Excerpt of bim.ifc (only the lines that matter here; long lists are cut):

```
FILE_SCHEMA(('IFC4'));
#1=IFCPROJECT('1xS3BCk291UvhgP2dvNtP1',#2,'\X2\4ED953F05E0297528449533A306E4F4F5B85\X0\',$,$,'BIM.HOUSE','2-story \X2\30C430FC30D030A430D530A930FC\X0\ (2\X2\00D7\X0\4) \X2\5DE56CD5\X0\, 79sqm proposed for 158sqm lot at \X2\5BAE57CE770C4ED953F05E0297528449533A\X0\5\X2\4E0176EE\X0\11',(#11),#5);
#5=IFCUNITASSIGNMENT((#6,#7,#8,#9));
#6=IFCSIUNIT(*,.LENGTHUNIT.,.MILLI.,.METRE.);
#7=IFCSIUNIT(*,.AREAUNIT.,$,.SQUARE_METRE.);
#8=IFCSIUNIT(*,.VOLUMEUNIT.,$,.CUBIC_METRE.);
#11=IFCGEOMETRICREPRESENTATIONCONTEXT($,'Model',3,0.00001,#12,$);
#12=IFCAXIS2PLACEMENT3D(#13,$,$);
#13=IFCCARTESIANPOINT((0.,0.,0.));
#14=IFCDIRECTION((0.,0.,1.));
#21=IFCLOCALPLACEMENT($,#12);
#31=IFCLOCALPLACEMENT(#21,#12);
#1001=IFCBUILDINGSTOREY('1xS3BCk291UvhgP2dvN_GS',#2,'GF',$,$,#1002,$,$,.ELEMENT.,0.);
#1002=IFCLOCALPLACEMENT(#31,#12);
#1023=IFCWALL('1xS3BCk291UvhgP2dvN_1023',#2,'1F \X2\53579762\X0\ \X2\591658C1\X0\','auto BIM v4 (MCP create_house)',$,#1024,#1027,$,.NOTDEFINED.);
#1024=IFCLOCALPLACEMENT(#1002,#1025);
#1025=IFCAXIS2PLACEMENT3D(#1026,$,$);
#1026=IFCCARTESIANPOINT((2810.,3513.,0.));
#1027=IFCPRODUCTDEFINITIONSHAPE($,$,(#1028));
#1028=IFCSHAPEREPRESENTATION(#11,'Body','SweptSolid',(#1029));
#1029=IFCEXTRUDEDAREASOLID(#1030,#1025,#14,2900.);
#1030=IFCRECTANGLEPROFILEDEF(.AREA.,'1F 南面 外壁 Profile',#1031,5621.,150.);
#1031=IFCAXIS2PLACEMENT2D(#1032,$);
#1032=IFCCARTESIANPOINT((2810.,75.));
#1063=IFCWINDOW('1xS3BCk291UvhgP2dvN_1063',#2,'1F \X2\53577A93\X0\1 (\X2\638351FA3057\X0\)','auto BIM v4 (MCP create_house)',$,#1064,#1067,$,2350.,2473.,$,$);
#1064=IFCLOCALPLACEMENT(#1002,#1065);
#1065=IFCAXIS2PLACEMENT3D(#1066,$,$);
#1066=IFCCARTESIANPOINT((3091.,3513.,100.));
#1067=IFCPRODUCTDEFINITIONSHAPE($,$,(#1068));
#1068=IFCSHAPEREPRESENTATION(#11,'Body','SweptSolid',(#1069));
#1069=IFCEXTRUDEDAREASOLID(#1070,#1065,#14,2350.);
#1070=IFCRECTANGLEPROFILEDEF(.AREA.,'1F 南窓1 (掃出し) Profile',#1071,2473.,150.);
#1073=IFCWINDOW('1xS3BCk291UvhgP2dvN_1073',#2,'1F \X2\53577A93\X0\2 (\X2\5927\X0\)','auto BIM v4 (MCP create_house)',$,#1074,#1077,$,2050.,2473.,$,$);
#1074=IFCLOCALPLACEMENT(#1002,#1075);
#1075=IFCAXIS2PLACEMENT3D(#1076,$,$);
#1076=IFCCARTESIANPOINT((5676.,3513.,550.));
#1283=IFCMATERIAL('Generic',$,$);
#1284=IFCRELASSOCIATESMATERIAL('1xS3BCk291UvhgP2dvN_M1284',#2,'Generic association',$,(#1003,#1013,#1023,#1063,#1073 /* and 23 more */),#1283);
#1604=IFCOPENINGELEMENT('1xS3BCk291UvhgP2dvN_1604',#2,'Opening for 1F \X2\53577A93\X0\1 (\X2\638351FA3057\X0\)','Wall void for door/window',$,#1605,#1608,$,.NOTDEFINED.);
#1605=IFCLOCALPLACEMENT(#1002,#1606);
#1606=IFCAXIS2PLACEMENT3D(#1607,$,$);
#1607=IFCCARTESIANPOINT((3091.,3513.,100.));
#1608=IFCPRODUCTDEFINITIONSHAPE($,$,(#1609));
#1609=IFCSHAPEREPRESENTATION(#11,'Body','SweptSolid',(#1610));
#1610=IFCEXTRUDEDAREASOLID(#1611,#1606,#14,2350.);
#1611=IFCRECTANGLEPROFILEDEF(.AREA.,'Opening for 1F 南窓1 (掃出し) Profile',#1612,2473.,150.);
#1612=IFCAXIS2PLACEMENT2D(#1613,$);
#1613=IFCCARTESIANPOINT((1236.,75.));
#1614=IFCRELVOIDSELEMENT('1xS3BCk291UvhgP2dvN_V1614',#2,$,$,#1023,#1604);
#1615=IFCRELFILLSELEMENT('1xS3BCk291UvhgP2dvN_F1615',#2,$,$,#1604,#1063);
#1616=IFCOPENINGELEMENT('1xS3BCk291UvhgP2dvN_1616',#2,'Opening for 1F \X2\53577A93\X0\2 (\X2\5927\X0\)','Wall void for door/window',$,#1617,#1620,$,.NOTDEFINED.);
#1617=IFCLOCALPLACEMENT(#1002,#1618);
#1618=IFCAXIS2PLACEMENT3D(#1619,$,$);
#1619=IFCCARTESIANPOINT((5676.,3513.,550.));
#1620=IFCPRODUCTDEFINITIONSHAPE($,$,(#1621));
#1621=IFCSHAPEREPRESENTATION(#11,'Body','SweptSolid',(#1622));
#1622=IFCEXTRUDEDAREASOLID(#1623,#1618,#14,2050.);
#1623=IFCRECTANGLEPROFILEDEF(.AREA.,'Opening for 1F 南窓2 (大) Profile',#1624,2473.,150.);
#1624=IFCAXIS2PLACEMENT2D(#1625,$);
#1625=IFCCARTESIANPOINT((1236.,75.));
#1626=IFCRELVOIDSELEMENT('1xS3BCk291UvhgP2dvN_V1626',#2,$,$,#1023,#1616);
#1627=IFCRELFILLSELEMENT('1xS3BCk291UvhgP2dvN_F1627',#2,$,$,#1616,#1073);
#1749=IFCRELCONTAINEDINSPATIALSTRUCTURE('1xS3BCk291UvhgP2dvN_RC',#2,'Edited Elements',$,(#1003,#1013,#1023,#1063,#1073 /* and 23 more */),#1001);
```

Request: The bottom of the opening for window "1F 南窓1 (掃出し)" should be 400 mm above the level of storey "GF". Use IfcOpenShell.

```python
import numpy as np
import ifcopenshell
import ifcopenshell.api.geometry
import ifcopenshell.geom
import ifcopenshell.util.element
import ifcopenshell.util.placement
import ifcopenshell.util.shape
import ifcopenshell.util.unit

model = ifcopenshell.open("bim.ifc")
unit_scale = ifcopenshell.util.unit.calculate_unit_scale(model)

window = model.by_id(1063)
opening = window.FillsVoids[0].RelatingOpeningElement
storey = ifcopenshell.util.element.get_container(window, ifc_class="IfcBuildingStorey")
level = ifcopenshell.util.placement.get_local_placement(storey.ObjectPlacement)[2, 3]

# The opening's origin need not be at the sill, so measure its lowest point.
shape = ifcopenshell.geom.create_shape(ifcopenshell.geom.settings(), opening)
bottom = ifcopenshell.util.shape.get_shape_bottom_elevation(shape, shape.geometry) / unit_scale
dz = level + 400.0 - bottom

shift = np.array([0.0, 0.0, dz])
# The window is not placed relative to its opening, so move both.
for product in (opening, window):
    matrix = ifcopenshell.util.placement.get_local_placement(product.ObjectPlacement)
    matrix[:3, 3] += shift
    ifcopenshell.api.geometry.edit_object_placement(model, product=product, matrix=matrix, is_si=False)

print(f"moved by {dz * unit_scale:+.3f} m")

model.write("bim_v2.ifc")
```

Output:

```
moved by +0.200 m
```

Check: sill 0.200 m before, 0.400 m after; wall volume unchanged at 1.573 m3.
